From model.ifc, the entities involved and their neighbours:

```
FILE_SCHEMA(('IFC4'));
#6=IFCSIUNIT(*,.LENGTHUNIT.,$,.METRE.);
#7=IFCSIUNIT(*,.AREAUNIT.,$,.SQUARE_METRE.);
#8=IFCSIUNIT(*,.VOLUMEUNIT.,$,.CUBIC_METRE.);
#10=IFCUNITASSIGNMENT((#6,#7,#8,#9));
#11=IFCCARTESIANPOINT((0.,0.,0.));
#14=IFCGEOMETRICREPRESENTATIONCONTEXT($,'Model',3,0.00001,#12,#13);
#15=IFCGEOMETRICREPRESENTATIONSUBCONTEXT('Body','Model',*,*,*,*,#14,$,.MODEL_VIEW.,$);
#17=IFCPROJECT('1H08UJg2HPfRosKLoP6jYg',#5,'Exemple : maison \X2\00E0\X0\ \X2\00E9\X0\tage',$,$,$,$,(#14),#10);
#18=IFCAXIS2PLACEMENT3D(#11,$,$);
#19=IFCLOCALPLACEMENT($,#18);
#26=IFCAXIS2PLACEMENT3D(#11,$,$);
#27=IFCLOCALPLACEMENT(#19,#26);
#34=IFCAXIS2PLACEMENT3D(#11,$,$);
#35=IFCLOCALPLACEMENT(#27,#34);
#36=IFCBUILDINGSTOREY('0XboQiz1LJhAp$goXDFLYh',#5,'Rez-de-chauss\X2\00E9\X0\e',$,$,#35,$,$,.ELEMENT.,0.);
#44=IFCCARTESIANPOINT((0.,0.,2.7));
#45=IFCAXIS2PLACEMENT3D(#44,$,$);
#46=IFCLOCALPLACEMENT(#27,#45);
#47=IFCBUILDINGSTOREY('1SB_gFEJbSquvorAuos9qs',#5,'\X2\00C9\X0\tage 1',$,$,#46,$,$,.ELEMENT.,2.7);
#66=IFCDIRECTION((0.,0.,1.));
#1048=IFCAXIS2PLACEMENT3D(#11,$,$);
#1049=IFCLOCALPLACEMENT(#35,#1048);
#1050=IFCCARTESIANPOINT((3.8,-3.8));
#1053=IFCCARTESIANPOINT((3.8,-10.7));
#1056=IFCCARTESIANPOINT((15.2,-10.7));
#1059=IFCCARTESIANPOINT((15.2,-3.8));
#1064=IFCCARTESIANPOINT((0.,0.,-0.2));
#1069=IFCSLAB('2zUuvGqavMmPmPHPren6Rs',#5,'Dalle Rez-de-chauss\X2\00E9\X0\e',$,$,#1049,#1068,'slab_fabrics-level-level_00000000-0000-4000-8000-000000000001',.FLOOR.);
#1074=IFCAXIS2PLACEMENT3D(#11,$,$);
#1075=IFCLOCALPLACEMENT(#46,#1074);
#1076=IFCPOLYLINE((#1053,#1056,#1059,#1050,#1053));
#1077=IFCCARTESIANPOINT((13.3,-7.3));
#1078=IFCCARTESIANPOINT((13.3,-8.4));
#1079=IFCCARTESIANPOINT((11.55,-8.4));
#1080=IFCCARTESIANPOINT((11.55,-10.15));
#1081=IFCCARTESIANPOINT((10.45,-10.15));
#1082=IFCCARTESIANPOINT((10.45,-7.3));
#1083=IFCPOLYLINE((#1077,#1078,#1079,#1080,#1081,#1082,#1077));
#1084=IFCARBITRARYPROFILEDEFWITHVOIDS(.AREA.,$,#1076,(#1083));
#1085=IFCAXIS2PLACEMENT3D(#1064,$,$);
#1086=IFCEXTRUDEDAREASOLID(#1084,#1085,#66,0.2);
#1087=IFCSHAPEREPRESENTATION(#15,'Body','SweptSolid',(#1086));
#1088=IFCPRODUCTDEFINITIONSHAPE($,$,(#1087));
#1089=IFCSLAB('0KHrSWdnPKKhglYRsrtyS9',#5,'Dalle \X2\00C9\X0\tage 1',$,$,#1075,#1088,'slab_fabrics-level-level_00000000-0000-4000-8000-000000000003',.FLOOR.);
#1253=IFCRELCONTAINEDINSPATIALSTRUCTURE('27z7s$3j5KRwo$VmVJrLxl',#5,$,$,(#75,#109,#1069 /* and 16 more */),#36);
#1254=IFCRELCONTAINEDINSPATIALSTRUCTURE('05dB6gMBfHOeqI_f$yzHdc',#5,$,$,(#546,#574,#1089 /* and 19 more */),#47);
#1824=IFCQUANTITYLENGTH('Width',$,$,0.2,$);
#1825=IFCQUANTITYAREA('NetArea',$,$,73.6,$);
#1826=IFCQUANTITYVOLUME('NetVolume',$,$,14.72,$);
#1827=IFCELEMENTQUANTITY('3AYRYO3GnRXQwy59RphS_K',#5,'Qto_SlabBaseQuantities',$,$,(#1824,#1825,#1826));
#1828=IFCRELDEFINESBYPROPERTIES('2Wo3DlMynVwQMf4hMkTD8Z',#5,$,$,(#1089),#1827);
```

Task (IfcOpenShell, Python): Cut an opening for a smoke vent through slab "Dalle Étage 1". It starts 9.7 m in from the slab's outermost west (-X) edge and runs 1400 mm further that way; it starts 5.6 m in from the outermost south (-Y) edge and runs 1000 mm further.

```python
import numpy as np
import ifcopenshell
import ifcopenshell.api.feature
import ifcopenshell.api.geometry
import ifcopenshell.api.pset
import ifcopenshell.api.root
import ifcopenshell.geom
import ifcopenshell.util.element
import ifcopenshell.util.placement
import ifcopenshell.util.representation
import ifcopenshell.util.shape
import ifcopenshell.util.unit

model = ifcopenshell.open("model.ifc")
unit_scale = ifcopenshell.util.unit.calculate_unit_scale(model)
area_scale = ifcopenshell.util.unit.calculate_unit_scale(model, "AREAUNIT")
volume_scale = ifcopenshell.util.unit.calculate_unit_scale(model, "VOLUMEUNIT")
settings = ifcopenshell.geom.settings()


def volume(element):
    """Net volume in cubic metres, openings subtracted."""
    shape = ifcopenshell.geom.create_shape(settings, element)
    return ifcopenshell.util.shape.get_volume(shape.geometry)


slab = model.by_guid("0KHrSWdnPKKhglYRsrtyS9")
before = volume(slab)

# Extent in the slab's own axes, in metres. The edges named are its -X and -Y sides.
slab_shape = ifcopenshell.geom.create_shape(settings, slab)
vertices = ifcopenshell.util.shape.get_vertices(slab_shape.geometry)
x_min, y_min, bottom = vertices.min(axis=0)
top = vertices[:, 2].max()

opening = ifcopenshell.api.root.create_entity(model, ifc_class="IfcOpeningElement", name="Smoke vent opening", predefined_type="OPENING")
context = ifcopenshell.util.representation.get_context(model, "Model", "Body", "MODEL_VIEW")
width, depth = 1.4, 1
outline = [(0.0, 0.0), (width, 0.0), (width, depth), (0.0, depth), (0.0, 0.0)]
# Overshoot both faces by 50 mm so the cut is clean.
shape = ifcopenshell.api.geometry.add_slab_representation(
    model, context=context, depth=top - bottom + 0.1, polyline=outline
)
ifcopenshell.api.geometry.assign_representation(model, product=opening, representation=shape)

matrix = ifcopenshell.util.placement.get_local_placement(slab.ObjectPlacement)
matrix[:, 3] = matrix @ np.append(np.array([x_min + 9.7, y_min + 5.6, bottom - 0.05]) / unit_scale, 1.0)
ifcopenshell.api.geometry.edit_object_placement(model, product=opening, matrix=matrix, is_si=False)
ifcopenshell.api.feature.add_feature(model, feature=opening, element=slab)

after = volume(slab)

# Update the slab's stored quantities.
qto = model.by_id(ifcopenshell.util.element.get_pset(slab, "Qto_SlabBaseQuantities", should_inherit=False)["id"])
ifcopenshell.api.pset.edit_qto(model, qto=qto, properties={
    "NetArea": after / (top - bottom) / area_scale,
    "NetVolume": after / volume_scale,
})

print(f"slab volume {before:.3f} -> {after:.3f} m3")

model.write("model_rev.ifc")
```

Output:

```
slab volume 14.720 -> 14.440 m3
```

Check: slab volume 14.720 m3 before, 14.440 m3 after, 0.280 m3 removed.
